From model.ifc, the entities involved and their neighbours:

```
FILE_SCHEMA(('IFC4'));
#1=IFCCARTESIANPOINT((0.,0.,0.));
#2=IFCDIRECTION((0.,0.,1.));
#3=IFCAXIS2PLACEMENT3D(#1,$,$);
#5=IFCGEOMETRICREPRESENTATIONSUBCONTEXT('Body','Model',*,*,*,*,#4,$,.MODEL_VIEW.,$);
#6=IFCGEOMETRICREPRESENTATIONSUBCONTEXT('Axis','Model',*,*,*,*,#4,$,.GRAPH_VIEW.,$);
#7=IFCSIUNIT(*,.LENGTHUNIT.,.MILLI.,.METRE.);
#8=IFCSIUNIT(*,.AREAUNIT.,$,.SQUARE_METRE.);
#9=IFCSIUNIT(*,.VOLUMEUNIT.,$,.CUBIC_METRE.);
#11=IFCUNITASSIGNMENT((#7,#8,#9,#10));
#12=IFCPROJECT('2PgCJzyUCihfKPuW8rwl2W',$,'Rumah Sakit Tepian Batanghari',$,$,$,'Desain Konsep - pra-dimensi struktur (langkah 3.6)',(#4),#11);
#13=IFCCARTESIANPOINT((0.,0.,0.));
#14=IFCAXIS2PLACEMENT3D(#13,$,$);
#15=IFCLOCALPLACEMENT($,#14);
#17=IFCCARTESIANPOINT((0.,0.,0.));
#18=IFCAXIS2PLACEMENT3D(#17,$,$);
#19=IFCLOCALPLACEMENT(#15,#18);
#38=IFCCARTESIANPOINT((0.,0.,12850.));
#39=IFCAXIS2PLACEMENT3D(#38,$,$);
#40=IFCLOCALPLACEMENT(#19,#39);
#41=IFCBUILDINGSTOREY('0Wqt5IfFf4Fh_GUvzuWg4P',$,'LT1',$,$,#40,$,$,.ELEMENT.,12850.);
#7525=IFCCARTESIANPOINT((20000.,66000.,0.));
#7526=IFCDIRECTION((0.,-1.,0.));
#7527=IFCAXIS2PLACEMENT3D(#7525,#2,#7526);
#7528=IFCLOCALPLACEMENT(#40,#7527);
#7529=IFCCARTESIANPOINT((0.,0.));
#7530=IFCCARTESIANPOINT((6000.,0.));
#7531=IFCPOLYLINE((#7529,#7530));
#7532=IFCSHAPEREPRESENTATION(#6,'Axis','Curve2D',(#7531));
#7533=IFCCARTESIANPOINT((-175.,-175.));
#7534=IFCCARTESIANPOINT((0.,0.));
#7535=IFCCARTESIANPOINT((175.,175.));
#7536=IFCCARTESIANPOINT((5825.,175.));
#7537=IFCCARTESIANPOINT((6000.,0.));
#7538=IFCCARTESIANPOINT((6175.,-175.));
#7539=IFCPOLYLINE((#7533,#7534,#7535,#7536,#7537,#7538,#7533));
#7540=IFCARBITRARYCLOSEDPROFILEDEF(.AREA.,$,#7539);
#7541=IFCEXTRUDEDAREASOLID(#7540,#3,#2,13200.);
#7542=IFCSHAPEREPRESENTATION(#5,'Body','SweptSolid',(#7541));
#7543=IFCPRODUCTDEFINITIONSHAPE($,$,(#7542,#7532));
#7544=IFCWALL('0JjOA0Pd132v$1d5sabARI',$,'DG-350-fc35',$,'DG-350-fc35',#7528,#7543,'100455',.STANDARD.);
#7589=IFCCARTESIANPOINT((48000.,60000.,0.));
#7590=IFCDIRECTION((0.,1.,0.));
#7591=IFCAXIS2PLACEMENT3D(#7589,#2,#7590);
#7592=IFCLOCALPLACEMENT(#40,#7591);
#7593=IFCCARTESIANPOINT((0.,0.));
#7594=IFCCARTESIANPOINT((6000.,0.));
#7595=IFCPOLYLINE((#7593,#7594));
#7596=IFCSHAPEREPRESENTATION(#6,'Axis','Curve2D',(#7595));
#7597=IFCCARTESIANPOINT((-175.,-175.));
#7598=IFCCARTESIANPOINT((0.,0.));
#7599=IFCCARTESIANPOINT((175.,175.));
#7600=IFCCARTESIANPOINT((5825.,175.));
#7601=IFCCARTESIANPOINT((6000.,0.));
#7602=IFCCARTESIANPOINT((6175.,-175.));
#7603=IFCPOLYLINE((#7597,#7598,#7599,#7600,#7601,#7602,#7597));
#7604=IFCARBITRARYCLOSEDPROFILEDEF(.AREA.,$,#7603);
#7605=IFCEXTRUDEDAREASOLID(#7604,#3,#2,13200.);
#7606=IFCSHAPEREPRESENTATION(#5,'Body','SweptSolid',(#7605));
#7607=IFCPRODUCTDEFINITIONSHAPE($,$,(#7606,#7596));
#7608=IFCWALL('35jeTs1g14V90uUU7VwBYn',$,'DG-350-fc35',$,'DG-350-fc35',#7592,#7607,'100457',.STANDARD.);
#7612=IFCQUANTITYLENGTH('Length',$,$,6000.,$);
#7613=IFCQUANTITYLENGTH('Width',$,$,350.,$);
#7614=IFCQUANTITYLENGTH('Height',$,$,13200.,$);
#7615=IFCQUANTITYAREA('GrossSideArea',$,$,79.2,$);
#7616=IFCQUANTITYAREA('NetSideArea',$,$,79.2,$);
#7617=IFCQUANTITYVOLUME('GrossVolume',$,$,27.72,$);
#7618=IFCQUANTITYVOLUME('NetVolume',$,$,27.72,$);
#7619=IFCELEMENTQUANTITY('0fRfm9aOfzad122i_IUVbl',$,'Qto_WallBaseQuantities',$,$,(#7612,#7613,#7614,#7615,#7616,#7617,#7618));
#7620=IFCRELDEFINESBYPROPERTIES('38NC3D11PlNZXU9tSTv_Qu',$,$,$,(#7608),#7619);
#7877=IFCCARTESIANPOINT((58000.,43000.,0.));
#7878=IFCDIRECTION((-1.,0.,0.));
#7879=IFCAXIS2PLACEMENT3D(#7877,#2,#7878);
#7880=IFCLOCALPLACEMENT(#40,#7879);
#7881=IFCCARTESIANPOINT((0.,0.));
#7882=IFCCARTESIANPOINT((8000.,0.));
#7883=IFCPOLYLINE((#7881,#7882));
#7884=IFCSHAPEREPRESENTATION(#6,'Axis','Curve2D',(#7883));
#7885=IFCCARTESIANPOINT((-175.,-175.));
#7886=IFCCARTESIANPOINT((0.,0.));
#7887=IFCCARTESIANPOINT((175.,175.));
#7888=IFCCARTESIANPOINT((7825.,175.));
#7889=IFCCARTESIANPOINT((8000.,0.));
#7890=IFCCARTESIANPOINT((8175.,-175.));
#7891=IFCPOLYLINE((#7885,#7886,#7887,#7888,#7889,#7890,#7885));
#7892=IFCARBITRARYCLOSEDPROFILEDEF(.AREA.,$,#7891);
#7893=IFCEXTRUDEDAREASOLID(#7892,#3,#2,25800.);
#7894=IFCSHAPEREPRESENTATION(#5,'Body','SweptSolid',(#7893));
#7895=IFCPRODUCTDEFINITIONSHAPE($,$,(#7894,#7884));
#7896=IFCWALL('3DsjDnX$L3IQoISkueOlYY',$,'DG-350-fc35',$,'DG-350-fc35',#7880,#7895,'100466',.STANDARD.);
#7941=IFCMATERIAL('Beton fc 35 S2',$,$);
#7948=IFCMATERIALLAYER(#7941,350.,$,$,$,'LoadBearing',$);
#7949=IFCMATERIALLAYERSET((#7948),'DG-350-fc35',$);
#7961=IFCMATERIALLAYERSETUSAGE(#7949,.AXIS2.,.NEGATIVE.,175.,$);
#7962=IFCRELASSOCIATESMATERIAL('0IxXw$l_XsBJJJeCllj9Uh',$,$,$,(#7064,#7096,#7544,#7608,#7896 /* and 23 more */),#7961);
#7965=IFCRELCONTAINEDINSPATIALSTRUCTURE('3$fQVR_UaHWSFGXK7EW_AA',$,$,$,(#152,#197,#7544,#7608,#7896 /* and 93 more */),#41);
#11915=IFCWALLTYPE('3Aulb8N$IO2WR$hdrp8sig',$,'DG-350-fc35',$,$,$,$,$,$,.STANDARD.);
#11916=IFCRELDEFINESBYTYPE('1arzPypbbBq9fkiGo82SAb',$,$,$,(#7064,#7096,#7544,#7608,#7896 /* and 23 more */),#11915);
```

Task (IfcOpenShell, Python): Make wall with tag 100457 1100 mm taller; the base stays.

```python
import ifcopenshell
import ifcopenshell.api.pset
import ifcopenshell.geom
import ifcopenshell.util.element
import ifcopenshell.util.representation
import ifcopenshell.util.shape
import ifcopenshell.util.unit

model = ifcopenshell.open("model.ifc")
unit_scale = ifcopenshell.util.unit.calculate_unit_scale(model)
area_scale = ifcopenshell.util.unit.calculate_unit_scale(model, "AREAUNIT")
volume_scale = ifcopenshell.util.unit.calculate_unit_scale(model, "VOLUMEUNIT")
settings = ifcopenshell.geom.settings()


def volume(element):
    """Net volume in cubic metres, openings subtracted."""
    shape = ifcopenshell.geom.create_shape(settings, element)
    return ifcopenshell.util.shape.get_volume(shape.geometry)


wall = model.by_guid("35jeTs1g14V90uUU7VwBYn")
before = volume(wall)

body = ifcopenshell.util.representation.get_representation(wall, "Model", "Body")
solid = body.Items[0]
old_height = solid.Depth
solid.Depth += 1100.0
after = volume(wall)
thickness = 0.35  # wall thickness in metres

# Update the stored height, areas and volumes.
qto = model.by_id(ifcopenshell.util.element.get_pset(wall, "Qto_WallBaseQuantities", should_inherit=False)["id"])
ifcopenshell.api.pset.edit_qto(model, qto=qto, properties={
    "Height": solid.Depth,
    "GrossSideArea": ifcopenshell.util.element.get_pset(wall, "Qto_WallBaseQuantities", "GrossSideArea") * solid.Depth / old_height,
    "NetSideArea": after / thickness / area_scale,
    "GrossVolume": ifcopenshell.util.element.get_pset(wall, "Qto_WallBaseQuantities", "GrossVolume") * solid.Depth / old_height,
    "NetVolume": after / volume_scale,
})

print(f"height {old_height:g} -> {solid.Depth:g}, volume {before:.3f} -> {after:.3f} m3")

model.write("model_rev.ifc")
```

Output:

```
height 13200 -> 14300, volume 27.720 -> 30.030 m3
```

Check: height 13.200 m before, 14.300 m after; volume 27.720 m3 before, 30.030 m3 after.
